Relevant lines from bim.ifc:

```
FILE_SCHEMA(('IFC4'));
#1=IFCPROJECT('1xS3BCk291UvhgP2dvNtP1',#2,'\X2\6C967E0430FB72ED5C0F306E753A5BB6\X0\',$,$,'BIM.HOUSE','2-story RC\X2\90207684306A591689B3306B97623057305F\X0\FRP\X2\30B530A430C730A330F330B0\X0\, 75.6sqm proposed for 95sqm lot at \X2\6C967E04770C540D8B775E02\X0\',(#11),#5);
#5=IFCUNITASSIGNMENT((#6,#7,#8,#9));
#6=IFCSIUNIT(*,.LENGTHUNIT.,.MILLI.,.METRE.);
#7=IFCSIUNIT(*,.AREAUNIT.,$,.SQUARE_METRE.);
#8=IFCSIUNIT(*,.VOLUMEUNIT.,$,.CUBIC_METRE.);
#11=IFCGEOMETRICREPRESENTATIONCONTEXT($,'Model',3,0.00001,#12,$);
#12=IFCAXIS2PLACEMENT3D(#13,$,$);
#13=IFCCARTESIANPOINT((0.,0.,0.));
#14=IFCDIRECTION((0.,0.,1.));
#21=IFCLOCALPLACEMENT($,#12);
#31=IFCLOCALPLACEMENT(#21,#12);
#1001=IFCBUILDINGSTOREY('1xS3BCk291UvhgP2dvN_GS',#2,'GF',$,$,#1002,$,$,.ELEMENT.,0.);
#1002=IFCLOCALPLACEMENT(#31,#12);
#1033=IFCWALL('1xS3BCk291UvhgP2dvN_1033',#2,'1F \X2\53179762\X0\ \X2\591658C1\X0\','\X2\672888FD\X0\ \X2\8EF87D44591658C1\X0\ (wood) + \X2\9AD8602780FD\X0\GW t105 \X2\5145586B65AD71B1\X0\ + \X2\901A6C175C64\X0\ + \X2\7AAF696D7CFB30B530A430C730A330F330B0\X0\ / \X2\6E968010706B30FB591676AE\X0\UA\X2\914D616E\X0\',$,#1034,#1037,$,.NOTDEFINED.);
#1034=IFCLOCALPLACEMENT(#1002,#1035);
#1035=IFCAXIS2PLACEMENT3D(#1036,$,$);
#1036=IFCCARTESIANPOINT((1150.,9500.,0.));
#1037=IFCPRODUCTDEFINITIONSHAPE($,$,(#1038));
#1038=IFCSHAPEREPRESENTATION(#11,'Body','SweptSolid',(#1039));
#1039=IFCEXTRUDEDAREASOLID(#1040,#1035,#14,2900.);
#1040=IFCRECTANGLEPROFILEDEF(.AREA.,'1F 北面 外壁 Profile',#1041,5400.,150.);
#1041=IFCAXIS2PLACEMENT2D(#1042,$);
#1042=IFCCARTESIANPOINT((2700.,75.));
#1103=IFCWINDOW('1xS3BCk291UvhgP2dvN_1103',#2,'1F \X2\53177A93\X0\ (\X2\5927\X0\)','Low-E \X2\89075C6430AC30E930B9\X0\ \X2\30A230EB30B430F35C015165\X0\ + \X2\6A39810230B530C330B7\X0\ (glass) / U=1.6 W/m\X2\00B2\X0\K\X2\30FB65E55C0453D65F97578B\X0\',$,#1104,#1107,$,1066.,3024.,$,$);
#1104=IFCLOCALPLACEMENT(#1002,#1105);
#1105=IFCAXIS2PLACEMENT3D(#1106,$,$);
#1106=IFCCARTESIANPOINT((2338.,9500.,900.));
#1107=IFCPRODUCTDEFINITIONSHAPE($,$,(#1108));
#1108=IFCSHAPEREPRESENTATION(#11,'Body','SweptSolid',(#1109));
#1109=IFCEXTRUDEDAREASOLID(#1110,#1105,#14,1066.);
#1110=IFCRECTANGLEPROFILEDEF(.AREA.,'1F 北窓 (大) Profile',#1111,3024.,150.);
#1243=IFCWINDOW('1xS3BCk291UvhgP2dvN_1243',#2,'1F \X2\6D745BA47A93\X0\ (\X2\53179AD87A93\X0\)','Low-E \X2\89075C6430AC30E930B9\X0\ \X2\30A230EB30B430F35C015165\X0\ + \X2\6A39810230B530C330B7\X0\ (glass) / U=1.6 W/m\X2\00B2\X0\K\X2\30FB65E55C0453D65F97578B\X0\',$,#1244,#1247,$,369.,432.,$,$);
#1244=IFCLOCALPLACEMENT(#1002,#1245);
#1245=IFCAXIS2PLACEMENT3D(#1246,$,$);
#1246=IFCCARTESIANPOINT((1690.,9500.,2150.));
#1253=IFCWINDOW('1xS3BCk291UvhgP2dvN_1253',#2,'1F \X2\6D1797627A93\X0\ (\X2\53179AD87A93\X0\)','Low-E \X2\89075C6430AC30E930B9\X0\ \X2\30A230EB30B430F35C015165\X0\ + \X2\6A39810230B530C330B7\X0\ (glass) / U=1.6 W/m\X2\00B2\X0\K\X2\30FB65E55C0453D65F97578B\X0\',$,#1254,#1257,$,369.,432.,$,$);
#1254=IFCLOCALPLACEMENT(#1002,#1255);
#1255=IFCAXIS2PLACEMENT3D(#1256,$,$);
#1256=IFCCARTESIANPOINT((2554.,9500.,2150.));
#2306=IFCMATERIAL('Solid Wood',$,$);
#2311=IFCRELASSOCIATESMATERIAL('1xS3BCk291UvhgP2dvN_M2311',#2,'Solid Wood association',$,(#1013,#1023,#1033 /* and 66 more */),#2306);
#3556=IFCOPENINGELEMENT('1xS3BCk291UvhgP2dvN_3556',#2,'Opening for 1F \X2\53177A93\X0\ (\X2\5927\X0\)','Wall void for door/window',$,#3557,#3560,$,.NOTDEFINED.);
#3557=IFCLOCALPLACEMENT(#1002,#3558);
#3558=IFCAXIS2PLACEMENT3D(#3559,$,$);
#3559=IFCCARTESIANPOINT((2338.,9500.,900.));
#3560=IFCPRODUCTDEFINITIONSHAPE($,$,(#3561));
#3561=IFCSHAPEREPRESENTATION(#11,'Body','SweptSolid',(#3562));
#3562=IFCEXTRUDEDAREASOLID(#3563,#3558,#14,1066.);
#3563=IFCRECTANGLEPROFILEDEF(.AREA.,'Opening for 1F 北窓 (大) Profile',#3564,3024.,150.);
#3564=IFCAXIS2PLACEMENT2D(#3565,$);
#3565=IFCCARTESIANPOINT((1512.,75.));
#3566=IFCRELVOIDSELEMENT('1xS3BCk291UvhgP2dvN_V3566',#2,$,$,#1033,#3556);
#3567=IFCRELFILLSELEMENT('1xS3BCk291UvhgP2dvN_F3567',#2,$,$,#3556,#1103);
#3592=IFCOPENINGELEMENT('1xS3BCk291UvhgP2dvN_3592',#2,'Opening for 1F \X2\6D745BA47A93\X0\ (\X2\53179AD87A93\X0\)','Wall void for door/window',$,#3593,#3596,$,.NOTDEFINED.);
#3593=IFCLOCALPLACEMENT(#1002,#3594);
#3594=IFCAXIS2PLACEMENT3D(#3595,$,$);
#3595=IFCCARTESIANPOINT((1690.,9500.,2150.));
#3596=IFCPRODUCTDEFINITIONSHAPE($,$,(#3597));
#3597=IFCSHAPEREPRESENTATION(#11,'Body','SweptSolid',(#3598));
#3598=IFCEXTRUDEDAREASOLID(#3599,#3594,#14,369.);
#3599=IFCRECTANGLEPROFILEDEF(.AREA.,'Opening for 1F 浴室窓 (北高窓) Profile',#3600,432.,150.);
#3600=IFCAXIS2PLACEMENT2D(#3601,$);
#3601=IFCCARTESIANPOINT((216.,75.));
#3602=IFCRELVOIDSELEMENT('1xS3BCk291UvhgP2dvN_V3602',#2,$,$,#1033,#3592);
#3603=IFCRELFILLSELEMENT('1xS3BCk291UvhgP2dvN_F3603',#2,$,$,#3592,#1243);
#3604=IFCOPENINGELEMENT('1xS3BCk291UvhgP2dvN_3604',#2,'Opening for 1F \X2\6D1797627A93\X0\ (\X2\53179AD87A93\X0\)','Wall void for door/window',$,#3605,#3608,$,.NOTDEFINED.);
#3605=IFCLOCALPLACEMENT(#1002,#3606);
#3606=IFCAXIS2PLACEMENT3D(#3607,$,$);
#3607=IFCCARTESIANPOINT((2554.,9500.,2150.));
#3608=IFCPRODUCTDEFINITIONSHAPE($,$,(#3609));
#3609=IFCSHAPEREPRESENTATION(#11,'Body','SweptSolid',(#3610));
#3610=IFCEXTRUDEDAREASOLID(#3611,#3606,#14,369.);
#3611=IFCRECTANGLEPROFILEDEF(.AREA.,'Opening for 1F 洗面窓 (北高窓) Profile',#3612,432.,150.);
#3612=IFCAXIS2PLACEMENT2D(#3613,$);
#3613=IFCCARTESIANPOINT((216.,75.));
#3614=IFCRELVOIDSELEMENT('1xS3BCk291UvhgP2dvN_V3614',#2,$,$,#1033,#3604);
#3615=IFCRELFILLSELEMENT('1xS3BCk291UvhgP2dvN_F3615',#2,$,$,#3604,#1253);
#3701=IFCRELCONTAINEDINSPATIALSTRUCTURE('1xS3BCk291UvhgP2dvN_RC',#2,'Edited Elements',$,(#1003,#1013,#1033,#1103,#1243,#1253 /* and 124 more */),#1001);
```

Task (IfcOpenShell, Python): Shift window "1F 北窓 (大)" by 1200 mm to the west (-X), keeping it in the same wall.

```python
import ifcopenshell
import ifcopenshell.api.geometry
import ifcopenshell.util.placement

model = ifcopenshell.open("bim.ifc")

window = model.by_id(1103)
opening = window.FillsVoids[0].RelatingOpeningElement
wall = opening.VoidsElements[0].RelatingBuildingElement

wall_matrix = ifcopenshell.util.placement.get_local_placement(wall.ObjectPlacement)
shift = wall_matrix[:3, 0] * -1200.0
before = ifcopenshell.util.placement.get_local_placement(window.ObjectPlacement)[:3, 3].copy()

# The window is not placed relative to its opening, so move both.
for product in (opening, window):
    matrix = ifcopenshell.util.placement.get_local_placement(product.ObjectPlacement)
    matrix[:3, 3] += shift
    ifcopenshell.api.geometry.edit_object_placement(model, product=product, matrix=matrix, is_si=False)

after = ifcopenshell.util.placement.get_local_placement(window.ObjectPlacement)[:3, 3]
print("window moved by", (after - before).round(3) + 0.0)

model.write("bim_v2.ifc")
```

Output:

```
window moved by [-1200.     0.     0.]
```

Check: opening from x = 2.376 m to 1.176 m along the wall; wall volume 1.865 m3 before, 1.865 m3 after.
